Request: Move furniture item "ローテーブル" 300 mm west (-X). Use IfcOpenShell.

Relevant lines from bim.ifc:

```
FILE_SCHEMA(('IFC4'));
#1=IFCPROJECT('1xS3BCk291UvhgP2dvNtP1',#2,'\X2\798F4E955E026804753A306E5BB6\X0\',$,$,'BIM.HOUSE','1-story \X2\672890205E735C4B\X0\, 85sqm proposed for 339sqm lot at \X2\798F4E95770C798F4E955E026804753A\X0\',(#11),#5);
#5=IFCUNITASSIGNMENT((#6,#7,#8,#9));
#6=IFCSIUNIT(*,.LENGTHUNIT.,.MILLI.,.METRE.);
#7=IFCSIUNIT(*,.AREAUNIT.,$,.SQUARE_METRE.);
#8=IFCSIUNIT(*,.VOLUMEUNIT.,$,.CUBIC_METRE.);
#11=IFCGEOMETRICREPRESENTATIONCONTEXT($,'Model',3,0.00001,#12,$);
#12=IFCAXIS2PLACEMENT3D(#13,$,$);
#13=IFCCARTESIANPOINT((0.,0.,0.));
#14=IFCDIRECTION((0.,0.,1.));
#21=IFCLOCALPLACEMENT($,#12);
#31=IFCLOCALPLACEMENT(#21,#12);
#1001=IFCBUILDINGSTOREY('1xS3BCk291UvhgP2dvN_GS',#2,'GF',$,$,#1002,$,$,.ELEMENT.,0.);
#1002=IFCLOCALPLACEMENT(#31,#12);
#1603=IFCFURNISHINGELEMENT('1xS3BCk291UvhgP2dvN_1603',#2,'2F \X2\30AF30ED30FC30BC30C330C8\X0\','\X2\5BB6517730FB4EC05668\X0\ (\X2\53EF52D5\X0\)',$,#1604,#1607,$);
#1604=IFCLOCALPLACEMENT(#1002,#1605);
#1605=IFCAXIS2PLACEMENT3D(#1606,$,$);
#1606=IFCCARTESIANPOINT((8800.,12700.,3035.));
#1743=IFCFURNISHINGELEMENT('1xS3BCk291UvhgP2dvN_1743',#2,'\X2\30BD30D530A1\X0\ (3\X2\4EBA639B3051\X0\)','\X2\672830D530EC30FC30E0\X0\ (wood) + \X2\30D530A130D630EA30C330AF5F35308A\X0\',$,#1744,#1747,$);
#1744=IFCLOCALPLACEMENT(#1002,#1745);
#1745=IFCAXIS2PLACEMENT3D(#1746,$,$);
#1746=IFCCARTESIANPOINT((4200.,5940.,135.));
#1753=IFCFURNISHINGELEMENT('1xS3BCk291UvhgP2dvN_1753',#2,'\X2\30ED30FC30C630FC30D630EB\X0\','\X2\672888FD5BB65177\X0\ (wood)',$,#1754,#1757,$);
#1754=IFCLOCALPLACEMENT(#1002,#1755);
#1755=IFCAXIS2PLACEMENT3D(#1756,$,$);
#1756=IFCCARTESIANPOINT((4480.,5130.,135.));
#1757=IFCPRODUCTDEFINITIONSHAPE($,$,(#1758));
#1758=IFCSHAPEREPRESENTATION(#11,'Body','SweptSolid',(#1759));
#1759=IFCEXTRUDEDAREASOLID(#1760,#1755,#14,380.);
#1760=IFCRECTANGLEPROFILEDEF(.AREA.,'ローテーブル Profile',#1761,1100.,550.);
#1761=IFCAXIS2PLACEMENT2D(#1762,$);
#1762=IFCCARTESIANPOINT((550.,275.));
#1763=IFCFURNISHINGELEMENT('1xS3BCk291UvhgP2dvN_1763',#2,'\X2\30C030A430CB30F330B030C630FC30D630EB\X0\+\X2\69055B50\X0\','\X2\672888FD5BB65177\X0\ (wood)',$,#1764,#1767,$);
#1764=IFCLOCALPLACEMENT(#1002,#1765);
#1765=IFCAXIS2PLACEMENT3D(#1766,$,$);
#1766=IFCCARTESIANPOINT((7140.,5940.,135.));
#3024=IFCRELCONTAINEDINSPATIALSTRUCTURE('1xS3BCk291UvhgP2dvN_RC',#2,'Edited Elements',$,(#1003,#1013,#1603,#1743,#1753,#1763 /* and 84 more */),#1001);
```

```python
import ifcopenshell
import ifcopenshell.api.geometry
import ifcopenshell.util.placement
import ifcopenshell.util.unit

model = ifcopenshell.open("bim.ifc")
unit_scale = ifcopenshell.util.unit.calculate_unit_scale(model)

item = model.by_guid("1xS3BCk291UvhgP2dvN_1753")
matrix = ifcopenshell.util.placement.get_local_placement(item.ObjectPlacement)
matrix[0, 3] -= 0.3 / unit_scale
ifcopenshell.api.geometry.edit_object_placement(model, product=item, matrix=matrix, is_si=False)

print(ifcopenshell.util.placement.get_local_placement(item.ObjectPlacement).round(3) + 0.0)

model.write("bim_v2.ifc")
```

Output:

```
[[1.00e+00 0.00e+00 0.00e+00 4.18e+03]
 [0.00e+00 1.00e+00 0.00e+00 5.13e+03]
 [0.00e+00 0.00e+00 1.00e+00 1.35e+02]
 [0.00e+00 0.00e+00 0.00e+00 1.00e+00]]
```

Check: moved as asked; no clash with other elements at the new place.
